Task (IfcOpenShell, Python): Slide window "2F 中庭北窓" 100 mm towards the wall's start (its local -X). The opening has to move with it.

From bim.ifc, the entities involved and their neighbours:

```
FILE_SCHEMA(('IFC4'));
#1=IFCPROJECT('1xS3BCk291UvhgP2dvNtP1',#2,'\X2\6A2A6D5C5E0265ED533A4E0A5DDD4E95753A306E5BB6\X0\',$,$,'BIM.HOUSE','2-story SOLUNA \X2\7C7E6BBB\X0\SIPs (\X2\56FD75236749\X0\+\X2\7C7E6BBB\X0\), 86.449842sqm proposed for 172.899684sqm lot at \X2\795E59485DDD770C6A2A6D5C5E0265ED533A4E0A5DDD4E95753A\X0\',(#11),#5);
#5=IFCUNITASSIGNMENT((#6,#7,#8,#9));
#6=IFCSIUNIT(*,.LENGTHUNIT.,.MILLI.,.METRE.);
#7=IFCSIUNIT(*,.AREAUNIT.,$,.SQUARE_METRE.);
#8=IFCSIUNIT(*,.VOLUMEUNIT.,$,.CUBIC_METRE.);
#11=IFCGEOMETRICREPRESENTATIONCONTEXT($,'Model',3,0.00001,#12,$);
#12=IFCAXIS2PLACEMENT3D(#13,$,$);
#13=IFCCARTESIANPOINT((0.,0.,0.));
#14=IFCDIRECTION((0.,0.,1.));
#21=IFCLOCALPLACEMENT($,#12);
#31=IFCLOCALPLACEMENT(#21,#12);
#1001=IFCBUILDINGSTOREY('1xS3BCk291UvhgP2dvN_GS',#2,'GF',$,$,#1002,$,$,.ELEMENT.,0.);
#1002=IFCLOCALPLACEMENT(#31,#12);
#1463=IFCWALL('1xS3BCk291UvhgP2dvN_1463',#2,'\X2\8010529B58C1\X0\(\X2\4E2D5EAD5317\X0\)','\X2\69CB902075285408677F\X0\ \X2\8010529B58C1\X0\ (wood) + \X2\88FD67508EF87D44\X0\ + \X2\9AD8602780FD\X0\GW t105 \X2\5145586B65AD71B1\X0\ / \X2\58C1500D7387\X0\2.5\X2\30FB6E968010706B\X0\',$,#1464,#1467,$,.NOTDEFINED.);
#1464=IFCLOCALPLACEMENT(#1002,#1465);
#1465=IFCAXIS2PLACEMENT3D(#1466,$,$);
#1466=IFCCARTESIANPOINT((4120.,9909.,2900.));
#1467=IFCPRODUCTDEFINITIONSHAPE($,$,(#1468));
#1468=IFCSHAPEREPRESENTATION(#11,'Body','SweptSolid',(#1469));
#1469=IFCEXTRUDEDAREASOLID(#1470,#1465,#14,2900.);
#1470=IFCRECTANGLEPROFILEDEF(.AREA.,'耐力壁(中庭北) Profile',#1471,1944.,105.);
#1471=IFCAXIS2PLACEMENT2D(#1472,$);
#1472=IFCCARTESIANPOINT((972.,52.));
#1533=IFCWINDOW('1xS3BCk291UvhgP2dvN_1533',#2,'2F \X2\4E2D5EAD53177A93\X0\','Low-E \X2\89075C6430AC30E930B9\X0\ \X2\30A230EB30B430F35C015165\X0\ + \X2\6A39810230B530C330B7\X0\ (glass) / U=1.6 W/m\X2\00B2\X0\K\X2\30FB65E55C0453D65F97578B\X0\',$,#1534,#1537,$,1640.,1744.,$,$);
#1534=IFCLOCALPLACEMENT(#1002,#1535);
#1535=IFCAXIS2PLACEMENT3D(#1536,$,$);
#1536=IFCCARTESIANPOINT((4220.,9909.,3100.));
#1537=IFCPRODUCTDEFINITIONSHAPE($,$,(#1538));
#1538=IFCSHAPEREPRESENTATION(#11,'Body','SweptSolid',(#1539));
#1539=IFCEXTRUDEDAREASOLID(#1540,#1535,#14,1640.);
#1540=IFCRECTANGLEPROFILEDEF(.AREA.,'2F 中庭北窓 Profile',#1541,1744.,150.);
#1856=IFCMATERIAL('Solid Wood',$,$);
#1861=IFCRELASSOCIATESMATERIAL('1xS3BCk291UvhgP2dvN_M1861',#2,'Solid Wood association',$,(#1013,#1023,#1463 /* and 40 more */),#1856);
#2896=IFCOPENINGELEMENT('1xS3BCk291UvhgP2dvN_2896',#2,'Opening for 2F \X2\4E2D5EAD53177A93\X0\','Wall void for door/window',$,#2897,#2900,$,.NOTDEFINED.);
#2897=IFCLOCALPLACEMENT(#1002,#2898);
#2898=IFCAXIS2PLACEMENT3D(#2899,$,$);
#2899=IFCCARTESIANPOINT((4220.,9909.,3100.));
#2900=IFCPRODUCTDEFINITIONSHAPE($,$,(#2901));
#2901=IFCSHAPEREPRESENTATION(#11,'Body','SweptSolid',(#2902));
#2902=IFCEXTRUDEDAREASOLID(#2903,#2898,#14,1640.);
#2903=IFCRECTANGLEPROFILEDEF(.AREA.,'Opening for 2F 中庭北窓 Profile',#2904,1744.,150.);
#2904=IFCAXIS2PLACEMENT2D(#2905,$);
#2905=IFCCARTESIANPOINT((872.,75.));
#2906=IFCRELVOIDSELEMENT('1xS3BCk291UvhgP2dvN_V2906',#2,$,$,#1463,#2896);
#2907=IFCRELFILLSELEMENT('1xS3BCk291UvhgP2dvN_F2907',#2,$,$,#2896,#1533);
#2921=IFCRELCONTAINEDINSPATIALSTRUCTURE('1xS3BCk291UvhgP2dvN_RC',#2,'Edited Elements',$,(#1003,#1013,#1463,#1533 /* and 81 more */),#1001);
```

```python
import ifcopenshell
import ifcopenshell.api.geometry
import ifcopenshell.util.placement

model = ifcopenshell.open("bim.ifc")

window = model.by_guid("1xS3BCk291UvhgP2dvN_1533")
opening = window.FillsVoids[0].RelatingOpeningElement
wall = opening.VoidsElements[0].RelatingBuildingElement

wall_matrix = ifcopenshell.util.placement.get_local_placement(wall.ObjectPlacement)
shift = wall_matrix[:3, 0] * -100.0
before = ifcopenshell.util.placement.get_local_placement(window.ObjectPlacement)[:3, 3].copy()

# The window is not placed relative to its opening, so move both.
for product in (opening, window):
    matrix = ifcopenshell.util.placement.get_local_placement(product.ObjectPlacement)
    matrix[:3, 3] += shift
    ifcopenshell.api.geometry.edit_object_placement(model, product=product, matrix=matrix, is_si=False)

after = ifcopenshell.util.placement.get_local_placement(window.ObjectPlacement)[:3, 3]
print("window moved by", (after - before).round(3) + 0.0)

model.write("bim_updated.ifc")
```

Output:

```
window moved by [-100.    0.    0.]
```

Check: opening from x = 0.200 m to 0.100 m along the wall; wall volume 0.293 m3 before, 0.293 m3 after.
